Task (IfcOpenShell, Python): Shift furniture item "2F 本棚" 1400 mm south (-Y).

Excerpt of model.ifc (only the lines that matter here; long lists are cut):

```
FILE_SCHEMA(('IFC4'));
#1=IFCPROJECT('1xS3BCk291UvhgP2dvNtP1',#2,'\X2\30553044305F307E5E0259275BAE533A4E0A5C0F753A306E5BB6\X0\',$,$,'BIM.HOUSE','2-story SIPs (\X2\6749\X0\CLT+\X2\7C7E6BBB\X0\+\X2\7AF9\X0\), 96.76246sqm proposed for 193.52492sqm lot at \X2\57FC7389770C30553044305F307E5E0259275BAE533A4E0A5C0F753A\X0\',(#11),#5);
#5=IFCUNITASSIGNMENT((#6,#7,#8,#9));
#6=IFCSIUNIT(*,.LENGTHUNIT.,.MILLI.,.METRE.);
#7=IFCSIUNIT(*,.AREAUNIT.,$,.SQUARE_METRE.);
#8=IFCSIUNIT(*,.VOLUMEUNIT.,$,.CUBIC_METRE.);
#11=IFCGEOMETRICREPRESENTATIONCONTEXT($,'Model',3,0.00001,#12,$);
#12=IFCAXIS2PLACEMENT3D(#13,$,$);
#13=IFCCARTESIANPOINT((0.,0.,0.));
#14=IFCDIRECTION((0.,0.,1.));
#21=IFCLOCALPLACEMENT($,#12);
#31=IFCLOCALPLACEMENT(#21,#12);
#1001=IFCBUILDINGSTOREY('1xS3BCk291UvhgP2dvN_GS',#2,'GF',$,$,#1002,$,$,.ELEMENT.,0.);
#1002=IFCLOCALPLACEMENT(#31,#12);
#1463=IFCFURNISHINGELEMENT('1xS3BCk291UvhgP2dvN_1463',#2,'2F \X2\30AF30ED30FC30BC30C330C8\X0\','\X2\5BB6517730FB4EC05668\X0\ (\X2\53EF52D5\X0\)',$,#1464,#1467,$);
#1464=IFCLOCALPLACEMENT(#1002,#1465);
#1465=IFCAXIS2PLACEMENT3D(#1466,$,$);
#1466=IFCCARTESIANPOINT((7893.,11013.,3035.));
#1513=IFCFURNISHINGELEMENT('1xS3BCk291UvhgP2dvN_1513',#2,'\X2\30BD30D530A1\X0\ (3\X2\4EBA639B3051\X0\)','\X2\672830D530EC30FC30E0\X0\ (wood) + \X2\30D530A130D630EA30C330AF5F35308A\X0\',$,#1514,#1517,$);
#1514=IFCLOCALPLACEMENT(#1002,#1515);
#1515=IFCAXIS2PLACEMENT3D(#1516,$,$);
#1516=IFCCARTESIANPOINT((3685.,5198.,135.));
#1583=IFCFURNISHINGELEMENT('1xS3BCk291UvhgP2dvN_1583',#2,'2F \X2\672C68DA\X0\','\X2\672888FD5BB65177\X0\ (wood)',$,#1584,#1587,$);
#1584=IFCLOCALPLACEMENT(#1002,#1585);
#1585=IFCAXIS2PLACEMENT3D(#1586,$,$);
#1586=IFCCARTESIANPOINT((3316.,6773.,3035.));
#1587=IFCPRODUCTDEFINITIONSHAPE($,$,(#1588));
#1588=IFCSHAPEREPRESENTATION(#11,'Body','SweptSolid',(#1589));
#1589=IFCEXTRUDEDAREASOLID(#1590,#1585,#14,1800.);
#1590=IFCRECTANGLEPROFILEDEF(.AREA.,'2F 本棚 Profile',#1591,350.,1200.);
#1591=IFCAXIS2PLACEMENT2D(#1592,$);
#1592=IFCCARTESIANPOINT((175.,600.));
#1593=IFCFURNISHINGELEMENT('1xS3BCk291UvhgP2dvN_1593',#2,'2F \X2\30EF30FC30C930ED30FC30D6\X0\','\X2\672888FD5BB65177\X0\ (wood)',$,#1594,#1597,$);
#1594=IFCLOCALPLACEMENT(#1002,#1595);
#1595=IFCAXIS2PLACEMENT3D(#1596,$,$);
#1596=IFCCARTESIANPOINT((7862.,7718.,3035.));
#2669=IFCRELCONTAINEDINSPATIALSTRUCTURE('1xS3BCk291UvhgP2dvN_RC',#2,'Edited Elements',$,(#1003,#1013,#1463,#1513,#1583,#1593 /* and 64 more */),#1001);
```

```python
import ifcopenshell
import ifcopenshell.api.geometry
import ifcopenshell.util.placement
import ifcopenshell.util.unit

model = ifcopenshell.open("model.ifc")
unit_scale = ifcopenshell.util.unit.calculate_unit_scale(model)

item = model.by_guid("1xS3BCk291UvhgP2dvN_1583")
matrix = ifcopenshell.util.placement.get_local_placement(item.ObjectPlacement)
matrix[1, 3] -= 1.4 / unit_scale
ifcopenshell.api.geometry.edit_object_placement(model, product=item, matrix=matrix, is_si=False)

print(ifcopenshell.util.placement.get_local_placement(item.ObjectPlacement).round(3) + 0.0)

model.write("model_updated.ifc")
```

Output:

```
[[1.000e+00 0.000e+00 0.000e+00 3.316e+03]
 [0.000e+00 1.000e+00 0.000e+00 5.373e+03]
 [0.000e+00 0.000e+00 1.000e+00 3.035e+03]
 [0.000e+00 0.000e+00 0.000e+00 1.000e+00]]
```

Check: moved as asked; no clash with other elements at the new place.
